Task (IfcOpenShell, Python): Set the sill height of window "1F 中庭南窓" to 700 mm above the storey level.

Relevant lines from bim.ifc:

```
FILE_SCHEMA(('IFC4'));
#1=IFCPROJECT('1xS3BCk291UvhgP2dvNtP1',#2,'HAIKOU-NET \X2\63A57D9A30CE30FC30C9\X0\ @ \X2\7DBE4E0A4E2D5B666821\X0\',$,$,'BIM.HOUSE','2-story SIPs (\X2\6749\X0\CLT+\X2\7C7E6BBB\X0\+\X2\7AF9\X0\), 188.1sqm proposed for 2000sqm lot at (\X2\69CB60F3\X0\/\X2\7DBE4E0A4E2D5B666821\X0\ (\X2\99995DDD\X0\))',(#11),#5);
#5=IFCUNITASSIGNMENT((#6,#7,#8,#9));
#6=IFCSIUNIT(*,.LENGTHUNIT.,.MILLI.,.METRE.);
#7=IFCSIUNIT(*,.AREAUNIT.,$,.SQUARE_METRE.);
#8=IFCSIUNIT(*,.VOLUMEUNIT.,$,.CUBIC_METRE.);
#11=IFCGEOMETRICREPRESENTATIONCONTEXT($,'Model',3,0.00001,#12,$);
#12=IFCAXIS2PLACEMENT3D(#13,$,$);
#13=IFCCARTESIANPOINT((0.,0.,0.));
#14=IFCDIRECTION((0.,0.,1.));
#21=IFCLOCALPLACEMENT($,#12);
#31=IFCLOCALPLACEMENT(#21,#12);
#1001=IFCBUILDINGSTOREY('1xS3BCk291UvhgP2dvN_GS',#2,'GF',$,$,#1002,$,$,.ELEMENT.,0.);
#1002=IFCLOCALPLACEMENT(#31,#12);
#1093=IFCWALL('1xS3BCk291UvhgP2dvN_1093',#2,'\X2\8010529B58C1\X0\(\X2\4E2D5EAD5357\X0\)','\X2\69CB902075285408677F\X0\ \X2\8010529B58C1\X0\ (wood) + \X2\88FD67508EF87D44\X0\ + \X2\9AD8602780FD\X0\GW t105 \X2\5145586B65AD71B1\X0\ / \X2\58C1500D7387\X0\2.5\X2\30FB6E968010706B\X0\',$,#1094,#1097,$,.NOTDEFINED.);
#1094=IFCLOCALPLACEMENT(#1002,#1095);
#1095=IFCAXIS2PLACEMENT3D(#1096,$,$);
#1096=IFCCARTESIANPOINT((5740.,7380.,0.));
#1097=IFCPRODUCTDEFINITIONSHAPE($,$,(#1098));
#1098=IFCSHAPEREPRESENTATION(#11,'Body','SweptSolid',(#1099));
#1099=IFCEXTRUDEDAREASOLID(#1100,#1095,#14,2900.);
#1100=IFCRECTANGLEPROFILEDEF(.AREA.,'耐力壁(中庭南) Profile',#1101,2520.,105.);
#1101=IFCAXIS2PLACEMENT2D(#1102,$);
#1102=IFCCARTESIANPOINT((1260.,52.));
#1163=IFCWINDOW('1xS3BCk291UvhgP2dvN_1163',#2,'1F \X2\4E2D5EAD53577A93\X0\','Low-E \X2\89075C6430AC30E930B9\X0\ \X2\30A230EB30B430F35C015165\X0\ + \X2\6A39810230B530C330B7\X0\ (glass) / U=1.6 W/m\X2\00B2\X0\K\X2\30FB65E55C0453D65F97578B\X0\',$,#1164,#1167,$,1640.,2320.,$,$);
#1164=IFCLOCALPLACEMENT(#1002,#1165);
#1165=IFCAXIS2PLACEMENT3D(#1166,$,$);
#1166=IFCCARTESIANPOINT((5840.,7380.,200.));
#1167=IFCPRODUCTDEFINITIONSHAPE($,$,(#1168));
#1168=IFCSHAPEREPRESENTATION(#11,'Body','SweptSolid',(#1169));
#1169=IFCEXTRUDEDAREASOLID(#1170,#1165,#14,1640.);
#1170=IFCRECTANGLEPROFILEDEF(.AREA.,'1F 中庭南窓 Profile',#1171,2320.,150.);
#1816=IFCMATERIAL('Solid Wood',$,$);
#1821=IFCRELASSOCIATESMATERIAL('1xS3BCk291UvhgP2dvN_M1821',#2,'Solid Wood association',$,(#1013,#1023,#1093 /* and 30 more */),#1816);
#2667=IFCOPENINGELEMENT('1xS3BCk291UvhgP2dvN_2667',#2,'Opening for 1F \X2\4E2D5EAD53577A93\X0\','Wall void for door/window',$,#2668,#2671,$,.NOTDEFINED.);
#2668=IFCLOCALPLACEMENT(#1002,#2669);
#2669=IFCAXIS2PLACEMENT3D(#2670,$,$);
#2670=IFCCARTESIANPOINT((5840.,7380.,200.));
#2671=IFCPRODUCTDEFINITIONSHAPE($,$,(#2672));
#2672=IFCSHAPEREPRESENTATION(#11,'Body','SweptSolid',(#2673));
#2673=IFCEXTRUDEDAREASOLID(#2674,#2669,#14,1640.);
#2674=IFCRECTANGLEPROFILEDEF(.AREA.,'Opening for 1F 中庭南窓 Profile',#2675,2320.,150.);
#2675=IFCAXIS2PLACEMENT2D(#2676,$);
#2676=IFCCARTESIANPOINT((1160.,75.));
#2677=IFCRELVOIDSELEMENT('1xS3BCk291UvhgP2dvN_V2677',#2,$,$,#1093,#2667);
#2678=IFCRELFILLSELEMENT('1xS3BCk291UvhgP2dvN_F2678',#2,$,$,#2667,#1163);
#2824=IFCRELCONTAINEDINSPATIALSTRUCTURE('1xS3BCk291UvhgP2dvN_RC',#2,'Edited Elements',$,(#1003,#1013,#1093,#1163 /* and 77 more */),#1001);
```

```python
import numpy as np
import ifcopenshell
import ifcopenshell.api.geometry
import ifcopenshell.geom
import ifcopenshell.util.element
import ifcopenshell.util.placement
import ifcopenshell.util.shape
import ifcopenshell.util.unit

model = ifcopenshell.open("bim.ifc")
unit_scale = ifcopenshell.util.unit.calculate_unit_scale(model)

window = model.by_guid("1xS3BCk291UvhgP2dvN_1163")
opening = window.FillsVoids[0].RelatingOpeningElement
storey = ifcopenshell.util.element.get_container(window, ifc_class="IfcBuildingStorey")
level = ifcopenshell.util.placement.get_local_placement(storey.ObjectPlacement)[2, 3]

# The opening's origin need not be at the sill, so measure its lowest point.
shape = ifcopenshell.geom.create_shape(ifcopenshell.geom.settings(), opening)
bottom = ifcopenshell.util.shape.get_shape_bottom_elevation(shape, shape.geometry) / unit_scale
dz = level + 0.7 / unit_scale - bottom

shift = np.array([0.0, 0.0, dz])
# The window is not placed relative to its opening, so move both.
for product in (opening, window):
    matrix = ifcopenshell.util.placement.get_local_placement(product.ObjectPlacement)
    matrix[:3, 3] += shift
    ifcopenshell.api.geometry.edit_object_placement(model, product=product, matrix=matrix, is_si=False)

print(f"moved by {dz * unit_scale:+.3f} m")

model.write("bim_updated.ifc")
```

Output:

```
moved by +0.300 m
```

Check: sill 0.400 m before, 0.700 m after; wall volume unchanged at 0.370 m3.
